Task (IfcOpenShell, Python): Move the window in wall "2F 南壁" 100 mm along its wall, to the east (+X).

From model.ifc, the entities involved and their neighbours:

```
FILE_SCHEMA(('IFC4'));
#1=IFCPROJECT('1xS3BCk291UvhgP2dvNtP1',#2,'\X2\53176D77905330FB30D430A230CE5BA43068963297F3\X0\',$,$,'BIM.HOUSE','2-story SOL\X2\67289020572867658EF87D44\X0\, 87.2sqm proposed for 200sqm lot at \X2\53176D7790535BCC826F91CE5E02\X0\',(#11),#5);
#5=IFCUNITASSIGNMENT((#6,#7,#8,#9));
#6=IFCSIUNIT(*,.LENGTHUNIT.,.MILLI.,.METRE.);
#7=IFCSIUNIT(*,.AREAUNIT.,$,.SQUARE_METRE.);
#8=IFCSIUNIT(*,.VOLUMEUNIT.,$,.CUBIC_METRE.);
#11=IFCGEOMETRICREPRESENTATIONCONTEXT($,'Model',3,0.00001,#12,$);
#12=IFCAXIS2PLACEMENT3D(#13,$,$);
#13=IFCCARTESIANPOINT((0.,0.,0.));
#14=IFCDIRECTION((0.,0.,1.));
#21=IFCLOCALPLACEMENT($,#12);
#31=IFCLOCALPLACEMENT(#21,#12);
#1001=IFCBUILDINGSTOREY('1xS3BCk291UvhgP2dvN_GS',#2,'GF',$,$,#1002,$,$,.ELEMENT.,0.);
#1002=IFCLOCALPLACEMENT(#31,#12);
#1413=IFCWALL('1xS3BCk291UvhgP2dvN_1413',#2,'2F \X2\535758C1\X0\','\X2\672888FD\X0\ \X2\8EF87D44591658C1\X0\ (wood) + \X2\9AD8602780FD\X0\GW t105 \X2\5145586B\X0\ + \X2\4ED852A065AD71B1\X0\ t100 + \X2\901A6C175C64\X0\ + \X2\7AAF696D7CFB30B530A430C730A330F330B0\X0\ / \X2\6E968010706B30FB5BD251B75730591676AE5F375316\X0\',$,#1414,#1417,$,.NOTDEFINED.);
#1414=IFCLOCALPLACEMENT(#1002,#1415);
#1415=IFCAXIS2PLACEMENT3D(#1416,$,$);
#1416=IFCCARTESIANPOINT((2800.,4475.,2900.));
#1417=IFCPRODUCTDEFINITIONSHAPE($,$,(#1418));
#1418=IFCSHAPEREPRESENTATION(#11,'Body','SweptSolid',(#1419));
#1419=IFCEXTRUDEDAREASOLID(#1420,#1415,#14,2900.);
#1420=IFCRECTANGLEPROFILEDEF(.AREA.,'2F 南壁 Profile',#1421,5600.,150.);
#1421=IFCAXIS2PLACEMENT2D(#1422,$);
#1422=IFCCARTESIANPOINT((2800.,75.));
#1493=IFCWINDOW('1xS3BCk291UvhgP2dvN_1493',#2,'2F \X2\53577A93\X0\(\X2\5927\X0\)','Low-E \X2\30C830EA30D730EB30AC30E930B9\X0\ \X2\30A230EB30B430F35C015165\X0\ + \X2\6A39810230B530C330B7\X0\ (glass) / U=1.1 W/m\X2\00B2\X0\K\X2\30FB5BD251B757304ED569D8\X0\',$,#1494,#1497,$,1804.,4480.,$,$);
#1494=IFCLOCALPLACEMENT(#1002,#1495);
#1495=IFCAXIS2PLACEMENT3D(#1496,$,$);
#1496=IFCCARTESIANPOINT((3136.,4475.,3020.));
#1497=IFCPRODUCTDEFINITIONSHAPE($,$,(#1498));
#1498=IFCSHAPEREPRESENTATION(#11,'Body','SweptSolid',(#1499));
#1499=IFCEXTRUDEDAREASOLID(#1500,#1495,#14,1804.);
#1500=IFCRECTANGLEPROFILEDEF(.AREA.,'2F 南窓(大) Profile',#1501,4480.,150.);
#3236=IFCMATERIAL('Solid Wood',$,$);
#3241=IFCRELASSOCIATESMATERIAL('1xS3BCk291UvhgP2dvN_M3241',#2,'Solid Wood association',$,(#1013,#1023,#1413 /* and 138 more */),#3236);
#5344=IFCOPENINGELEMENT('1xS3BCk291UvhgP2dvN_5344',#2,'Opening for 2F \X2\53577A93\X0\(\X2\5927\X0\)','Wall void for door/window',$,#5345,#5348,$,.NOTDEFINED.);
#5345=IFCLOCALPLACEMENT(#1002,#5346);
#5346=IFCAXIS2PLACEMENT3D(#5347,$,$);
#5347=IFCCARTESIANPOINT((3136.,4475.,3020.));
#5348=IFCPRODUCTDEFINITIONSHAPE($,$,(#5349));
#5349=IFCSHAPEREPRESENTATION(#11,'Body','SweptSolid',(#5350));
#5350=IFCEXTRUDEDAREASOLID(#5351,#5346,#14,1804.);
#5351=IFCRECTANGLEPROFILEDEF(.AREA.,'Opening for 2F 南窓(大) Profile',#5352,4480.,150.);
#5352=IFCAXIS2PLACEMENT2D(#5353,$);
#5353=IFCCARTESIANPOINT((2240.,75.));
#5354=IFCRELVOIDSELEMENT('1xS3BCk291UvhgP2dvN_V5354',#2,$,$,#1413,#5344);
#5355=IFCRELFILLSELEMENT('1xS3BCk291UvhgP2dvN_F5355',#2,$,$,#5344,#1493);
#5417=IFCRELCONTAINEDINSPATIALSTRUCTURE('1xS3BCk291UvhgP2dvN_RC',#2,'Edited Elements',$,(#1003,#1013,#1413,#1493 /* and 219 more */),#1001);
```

```python
import ifcopenshell
import ifcopenshell.api.geometry
import ifcopenshell.util.placement

model = ifcopenshell.open("model.ifc")

window = model.by_guid("1xS3BCk291UvhgP2dvN_1493")
opening = window.FillsVoids[0].RelatingOpeningElement
wall = opening.VoidsElements[0].RelatingBuildingElement

wall_matrix = ifcopenshell.util.placement.get_local_placement(wall.ObjectPlacement)
shift = wall_matrix[:3, 0] * 100.0
before = ifcopenshell.util.placement.get_local_placement(window.ObjectPlacement)[:3, 3].copy()

# The window is not placed relative to its opening, so move both.
for product in (opening, window):
    matrix = ifcopenshell.util.placement.get_local_placement(product.ObjectPlacement)
    matrix[:3, 3] += shift
    ifcopenshell.api.geometry.edit_object_placement(model, product=product, matrix=matrix, is_si=False)

after = ifcopenshell.util.placement.get_local_placement(window.ObjectPlacement)[:3, 3]
print("window moved by", (after - before).round(3) + 0.0)

model.write("model_edited.ifc")
```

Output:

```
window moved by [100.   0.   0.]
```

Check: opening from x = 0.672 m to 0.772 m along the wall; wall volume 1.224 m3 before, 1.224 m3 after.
